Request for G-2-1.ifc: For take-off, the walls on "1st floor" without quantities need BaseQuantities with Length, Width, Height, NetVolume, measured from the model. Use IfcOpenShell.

First a look at what the model holds.

```python
import ifcopenshell
import ifcopenshell.util.element
import ifcopenshell.util.unit

model = ifcopenshell.open("G-2-1.ifc")
print(model.schema)
for unit_type in ("LENGTHUNIT", "AREAUNIT", "VOLUMEUNIT"):
    print(unit_type, ifcopenshell.util.unit.calculate_unit_scale(model, unit_type))
storey = next(s for s in model.by_type("IfcBuildingStorey") if s.Name == "1st floor")
walls = [e for e in ifcopenshell.util.element.get_decomposition(storey) if e.is_a("IfcWall")]
for e in sorted(walls, key=lambda e: e.id()):
    print(e.id(), e.is_a(), e.Name, list(ifcopenshell.util.element.get_psets(e, qtos_only=True)), sep=" | ")
```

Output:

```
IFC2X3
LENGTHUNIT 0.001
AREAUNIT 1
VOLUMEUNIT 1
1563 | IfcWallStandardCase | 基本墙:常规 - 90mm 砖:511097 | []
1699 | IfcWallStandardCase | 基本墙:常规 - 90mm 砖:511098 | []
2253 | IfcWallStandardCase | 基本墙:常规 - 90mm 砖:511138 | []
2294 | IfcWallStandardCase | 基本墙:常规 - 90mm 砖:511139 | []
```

```python
import ifcopenshell
import ifcopenshell.api.pset
import ifcopenshell.geom
import ifcopenshell.util.element
import ifcopenshell.util.shape
import ifcopenshell.util.unit

model = ifcopenshell.open("G-2-1.ifc")
unit_scale = ifcopenshell.util.unit.calculate_unit_scale(model)
volume_scale = ifcopenshell.util.unit.calculate_unit_scale(model, "VOLUMEUNIT")
settings = ifcopenshell.geom.settings()

storey = next(s for s in model.by_type("IfcBuildingStorey") if s.Name == "1st floor")
walls = [e for e in ifcopenshell.util.element.get_decomposition(storey) if e.is_a("IfcWall")]

for e in sorted(walls, key=lambda e: e.id()):
    if ifcopenshell.util.element.get_psets(e, qtos_only=True, should_inherit=False):
        continue
    # Geometry comes back in metres, in the element's own axes.
    shape = ifcopenshell.geom.create_shape(settings, e)
    values = {
        "Length": ifcopenshell.util.shape.get_x(shape.geometry) / unit_scale,
        "Width": ifcopenshell.util.shape.get_y(shape.geometry) / unit_scale,
        "Height": ifcopenshell.util.shape.get_z(shape.geometry) / unit_scale,
        "NetVolume": ifcopenshell.util.shape.get_volume(shape.geometry) / volume_scale,
    }
    qto = ifcopenshell.api.pset.add_qto(model, product=e, name="BaseQuantities")
    ifcopenshell.api.pset.edit_qto(model, qto=qto, properties=values)
    print(e.id(), {k: round(v, 3) for k, v in values.items()})

model.write("G-2-1-out.ifc")
```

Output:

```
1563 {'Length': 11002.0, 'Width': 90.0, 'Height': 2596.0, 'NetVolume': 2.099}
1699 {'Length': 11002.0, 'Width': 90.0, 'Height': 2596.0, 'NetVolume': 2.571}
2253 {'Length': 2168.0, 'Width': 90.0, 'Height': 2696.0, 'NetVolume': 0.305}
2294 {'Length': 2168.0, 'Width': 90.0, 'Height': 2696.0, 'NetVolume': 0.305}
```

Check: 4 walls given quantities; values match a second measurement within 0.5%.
